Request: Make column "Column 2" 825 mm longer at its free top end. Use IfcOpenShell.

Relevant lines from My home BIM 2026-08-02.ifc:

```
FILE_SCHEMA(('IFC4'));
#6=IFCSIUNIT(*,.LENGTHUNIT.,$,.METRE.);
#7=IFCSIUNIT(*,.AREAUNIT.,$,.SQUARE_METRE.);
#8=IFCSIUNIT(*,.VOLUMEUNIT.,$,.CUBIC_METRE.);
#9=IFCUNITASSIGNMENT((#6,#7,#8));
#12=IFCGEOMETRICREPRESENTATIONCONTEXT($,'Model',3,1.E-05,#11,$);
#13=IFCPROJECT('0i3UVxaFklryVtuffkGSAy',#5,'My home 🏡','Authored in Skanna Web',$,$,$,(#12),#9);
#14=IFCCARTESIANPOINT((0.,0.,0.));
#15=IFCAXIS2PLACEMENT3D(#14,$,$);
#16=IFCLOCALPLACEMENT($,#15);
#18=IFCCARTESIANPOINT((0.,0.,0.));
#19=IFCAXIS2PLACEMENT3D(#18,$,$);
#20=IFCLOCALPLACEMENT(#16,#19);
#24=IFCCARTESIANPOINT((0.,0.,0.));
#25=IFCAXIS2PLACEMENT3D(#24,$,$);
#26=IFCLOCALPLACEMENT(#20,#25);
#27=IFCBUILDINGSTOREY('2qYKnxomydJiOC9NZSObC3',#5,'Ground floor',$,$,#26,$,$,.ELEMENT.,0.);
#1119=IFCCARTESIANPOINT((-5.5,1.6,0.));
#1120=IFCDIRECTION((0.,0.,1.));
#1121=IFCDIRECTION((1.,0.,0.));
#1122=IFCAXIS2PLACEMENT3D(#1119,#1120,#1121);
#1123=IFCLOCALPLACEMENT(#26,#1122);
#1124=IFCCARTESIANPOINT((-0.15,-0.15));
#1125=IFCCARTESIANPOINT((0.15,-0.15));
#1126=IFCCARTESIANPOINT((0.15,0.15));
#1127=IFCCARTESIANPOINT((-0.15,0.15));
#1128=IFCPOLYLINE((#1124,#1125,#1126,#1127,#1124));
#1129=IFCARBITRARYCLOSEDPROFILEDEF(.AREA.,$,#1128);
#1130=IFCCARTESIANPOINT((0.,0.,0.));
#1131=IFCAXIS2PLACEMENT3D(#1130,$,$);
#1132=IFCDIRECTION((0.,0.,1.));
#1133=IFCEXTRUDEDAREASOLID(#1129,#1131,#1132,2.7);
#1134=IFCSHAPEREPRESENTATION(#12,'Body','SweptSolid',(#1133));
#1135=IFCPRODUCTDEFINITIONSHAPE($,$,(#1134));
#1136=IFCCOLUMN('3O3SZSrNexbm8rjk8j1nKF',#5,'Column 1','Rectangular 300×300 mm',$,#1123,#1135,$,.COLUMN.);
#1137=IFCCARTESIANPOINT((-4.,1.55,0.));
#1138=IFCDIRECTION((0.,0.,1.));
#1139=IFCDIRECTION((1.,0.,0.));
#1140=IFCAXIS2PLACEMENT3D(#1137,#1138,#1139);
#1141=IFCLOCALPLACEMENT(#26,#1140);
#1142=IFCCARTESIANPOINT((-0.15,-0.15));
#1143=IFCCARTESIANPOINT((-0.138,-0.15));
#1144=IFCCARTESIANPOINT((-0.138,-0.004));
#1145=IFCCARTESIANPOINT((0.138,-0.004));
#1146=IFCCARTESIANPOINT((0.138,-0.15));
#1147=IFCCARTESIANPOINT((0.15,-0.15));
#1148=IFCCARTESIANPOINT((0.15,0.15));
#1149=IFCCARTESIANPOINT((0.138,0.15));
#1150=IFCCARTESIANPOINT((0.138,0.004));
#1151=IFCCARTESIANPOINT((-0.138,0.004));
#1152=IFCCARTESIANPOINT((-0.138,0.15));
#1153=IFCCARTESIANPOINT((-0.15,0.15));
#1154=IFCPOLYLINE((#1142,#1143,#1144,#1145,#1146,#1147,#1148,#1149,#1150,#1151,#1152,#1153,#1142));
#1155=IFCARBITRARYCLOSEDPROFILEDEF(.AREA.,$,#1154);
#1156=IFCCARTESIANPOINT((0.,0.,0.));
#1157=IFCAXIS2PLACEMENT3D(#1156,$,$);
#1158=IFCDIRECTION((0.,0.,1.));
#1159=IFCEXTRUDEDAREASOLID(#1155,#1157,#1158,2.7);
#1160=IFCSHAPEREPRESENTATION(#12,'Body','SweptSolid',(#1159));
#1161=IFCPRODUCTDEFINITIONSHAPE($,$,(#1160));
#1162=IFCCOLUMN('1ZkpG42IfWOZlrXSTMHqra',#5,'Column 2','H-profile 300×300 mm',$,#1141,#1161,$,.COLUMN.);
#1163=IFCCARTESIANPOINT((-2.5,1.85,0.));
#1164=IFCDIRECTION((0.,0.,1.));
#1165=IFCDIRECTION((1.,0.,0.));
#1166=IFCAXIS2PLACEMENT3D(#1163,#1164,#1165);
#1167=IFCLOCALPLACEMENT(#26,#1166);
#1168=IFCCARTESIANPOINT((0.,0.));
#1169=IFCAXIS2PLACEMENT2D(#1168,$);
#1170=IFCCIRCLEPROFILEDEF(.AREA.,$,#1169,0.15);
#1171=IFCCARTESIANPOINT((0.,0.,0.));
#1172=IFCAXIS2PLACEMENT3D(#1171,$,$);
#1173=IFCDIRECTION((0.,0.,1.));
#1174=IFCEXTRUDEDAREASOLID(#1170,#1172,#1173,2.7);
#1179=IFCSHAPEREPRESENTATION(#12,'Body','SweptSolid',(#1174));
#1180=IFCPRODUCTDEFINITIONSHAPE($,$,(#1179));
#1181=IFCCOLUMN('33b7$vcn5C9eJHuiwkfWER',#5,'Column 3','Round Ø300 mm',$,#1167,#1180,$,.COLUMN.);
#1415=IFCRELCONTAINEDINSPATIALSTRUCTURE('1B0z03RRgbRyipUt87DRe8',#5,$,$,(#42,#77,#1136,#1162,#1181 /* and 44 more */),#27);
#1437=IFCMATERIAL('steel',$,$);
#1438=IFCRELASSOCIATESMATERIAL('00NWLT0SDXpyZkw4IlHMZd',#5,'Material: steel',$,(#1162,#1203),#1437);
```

```python
import ifcopenshell
import ifcopenshell.util.unit

model = ifcopenshell.open("My home BIM 2026-08-02.ifc")
unit_scale = ifcopenshell.util.unit.calculate_unit_scale(model)

member = model.by_id(1162)
change = 0.825 / unit_scale

# The extrusion runs towards the end named, so only its depth changes.
body = next(r for r in member.Representation.Representations if r.RepresentationIdentifier == "Body")
solid = body.Items[0]
old_length = solid.Depth
solid.Depth += change

print(f"length {old_length:g} -> {solid.Depth:g}")

model.write("My home BIM 2026-08-02-out.ifc")
```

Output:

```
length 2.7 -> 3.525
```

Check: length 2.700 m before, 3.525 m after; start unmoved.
